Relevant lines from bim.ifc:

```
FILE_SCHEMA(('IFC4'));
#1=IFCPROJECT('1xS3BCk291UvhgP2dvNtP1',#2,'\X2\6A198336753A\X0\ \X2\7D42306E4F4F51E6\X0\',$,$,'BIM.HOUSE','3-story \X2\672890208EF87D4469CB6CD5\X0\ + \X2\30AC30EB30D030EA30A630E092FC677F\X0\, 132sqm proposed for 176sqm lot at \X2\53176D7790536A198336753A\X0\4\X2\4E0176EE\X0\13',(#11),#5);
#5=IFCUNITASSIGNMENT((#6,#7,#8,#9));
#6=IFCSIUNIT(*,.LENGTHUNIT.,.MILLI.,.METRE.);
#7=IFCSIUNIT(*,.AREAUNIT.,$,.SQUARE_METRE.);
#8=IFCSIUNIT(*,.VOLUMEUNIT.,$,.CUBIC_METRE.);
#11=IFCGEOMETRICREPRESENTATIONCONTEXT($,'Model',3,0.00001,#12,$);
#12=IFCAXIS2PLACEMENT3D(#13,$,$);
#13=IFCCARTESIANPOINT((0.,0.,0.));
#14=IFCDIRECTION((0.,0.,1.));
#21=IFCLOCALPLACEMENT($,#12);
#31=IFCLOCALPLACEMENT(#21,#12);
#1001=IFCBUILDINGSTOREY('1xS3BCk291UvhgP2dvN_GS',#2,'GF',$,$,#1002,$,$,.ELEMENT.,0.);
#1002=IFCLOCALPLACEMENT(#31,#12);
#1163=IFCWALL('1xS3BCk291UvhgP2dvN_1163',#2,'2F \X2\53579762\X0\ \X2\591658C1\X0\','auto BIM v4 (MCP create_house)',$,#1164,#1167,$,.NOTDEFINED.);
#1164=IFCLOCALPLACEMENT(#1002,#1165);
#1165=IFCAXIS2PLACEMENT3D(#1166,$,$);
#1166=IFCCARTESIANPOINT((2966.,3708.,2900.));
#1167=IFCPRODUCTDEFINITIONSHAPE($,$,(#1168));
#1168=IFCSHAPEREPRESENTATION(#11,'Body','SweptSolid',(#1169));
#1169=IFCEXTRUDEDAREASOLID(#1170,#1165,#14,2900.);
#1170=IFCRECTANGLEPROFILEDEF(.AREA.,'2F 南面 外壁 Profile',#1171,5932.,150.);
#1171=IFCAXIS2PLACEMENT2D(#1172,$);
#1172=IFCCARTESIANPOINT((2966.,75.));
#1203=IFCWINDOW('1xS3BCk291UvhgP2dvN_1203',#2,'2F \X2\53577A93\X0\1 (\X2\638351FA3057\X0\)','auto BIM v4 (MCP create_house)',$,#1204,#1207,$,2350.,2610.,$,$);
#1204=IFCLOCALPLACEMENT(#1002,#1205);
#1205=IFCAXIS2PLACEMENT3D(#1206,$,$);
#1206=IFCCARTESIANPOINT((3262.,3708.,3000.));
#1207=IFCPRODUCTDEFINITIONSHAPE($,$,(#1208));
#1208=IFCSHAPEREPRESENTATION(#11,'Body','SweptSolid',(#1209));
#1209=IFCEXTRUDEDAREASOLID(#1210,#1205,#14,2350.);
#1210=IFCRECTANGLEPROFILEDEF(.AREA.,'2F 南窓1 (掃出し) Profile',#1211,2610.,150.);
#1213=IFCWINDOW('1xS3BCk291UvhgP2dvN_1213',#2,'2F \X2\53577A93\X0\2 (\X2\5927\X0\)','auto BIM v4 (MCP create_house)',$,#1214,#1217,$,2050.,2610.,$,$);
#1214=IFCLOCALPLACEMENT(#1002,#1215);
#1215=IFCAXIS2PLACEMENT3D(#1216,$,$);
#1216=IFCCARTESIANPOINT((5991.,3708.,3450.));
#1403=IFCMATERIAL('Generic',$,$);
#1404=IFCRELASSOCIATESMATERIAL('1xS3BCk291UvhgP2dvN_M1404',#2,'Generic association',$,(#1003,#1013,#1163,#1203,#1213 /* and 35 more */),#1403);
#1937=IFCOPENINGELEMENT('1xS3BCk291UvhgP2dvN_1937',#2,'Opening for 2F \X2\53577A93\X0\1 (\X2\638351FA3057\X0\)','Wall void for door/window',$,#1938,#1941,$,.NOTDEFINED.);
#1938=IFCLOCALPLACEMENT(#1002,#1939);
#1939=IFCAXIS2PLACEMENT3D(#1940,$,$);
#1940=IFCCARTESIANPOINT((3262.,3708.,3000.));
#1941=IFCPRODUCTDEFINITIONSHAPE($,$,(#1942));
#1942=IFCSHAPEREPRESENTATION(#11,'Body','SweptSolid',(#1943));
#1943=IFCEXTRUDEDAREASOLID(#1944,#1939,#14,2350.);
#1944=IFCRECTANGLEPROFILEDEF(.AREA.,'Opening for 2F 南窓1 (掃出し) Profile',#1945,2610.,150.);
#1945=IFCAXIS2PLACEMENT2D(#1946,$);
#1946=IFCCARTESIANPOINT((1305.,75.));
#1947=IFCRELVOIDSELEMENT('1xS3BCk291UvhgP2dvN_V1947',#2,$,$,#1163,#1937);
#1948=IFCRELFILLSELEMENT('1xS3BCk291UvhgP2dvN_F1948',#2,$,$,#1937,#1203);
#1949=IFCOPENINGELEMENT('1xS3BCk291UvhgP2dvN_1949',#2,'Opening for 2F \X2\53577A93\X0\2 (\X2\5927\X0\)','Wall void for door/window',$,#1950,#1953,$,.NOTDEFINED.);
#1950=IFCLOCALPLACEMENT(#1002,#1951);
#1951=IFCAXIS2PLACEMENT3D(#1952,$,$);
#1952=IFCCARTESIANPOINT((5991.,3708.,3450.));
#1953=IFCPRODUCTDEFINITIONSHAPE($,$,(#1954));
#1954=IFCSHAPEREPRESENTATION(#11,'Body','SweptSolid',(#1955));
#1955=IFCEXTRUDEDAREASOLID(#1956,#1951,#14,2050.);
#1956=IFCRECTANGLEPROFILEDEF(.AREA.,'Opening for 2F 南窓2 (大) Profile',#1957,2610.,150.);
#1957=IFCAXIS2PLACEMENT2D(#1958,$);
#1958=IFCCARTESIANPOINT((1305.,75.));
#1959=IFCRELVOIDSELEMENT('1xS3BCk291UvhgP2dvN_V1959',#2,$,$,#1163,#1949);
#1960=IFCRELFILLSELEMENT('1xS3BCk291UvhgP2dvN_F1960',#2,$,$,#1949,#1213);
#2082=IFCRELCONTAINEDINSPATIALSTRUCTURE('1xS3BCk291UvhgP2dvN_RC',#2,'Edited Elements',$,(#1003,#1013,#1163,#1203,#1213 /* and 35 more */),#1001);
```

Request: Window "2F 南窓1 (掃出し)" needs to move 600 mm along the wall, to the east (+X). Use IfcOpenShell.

```python
import ifcopenshell
import ifcopenshell.api.geometry
import ifcopenshell.util.placement

model = ifcopenshell.open("bim.ifc")

window = model.by_guid("1xS3BCk291UvhgP2dvN_1203")
opening = window.FillsVoids[0].RelatingOpeningElement
wall = opening.VoidsElements[0].RelatingBuildingElement

wall_matrix = ifcopenshell.util.placement.get_local_placement(wall.ObjectPlacement)
shift = wall_matrix[:3, 0] * 600.0
before = ifcopenshell.util.placement.get_local_placement(window.ObjectPlacement)[:3, 3].copy()

# The window is not placed relative to its opening, so move both.
for product in (opening, window):
    matrix = ifcopenshell.util.placement.get_local_placement(product.ObjectPlacement)
    matrix[:3, 3] += shift
    ifcopenshell.api.geometry.edit_object_placement(model, product=product, matrix=matrix, is_si=False)

after = ifcopenshell.util.placement.get_local_placement(window.ObjectPlacement)[:3, 3]
print("window moved by", (after - before).round(3) + 0.0)

model.write("bim_edited.ifc")
```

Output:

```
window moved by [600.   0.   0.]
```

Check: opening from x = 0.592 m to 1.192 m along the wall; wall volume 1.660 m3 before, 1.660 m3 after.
